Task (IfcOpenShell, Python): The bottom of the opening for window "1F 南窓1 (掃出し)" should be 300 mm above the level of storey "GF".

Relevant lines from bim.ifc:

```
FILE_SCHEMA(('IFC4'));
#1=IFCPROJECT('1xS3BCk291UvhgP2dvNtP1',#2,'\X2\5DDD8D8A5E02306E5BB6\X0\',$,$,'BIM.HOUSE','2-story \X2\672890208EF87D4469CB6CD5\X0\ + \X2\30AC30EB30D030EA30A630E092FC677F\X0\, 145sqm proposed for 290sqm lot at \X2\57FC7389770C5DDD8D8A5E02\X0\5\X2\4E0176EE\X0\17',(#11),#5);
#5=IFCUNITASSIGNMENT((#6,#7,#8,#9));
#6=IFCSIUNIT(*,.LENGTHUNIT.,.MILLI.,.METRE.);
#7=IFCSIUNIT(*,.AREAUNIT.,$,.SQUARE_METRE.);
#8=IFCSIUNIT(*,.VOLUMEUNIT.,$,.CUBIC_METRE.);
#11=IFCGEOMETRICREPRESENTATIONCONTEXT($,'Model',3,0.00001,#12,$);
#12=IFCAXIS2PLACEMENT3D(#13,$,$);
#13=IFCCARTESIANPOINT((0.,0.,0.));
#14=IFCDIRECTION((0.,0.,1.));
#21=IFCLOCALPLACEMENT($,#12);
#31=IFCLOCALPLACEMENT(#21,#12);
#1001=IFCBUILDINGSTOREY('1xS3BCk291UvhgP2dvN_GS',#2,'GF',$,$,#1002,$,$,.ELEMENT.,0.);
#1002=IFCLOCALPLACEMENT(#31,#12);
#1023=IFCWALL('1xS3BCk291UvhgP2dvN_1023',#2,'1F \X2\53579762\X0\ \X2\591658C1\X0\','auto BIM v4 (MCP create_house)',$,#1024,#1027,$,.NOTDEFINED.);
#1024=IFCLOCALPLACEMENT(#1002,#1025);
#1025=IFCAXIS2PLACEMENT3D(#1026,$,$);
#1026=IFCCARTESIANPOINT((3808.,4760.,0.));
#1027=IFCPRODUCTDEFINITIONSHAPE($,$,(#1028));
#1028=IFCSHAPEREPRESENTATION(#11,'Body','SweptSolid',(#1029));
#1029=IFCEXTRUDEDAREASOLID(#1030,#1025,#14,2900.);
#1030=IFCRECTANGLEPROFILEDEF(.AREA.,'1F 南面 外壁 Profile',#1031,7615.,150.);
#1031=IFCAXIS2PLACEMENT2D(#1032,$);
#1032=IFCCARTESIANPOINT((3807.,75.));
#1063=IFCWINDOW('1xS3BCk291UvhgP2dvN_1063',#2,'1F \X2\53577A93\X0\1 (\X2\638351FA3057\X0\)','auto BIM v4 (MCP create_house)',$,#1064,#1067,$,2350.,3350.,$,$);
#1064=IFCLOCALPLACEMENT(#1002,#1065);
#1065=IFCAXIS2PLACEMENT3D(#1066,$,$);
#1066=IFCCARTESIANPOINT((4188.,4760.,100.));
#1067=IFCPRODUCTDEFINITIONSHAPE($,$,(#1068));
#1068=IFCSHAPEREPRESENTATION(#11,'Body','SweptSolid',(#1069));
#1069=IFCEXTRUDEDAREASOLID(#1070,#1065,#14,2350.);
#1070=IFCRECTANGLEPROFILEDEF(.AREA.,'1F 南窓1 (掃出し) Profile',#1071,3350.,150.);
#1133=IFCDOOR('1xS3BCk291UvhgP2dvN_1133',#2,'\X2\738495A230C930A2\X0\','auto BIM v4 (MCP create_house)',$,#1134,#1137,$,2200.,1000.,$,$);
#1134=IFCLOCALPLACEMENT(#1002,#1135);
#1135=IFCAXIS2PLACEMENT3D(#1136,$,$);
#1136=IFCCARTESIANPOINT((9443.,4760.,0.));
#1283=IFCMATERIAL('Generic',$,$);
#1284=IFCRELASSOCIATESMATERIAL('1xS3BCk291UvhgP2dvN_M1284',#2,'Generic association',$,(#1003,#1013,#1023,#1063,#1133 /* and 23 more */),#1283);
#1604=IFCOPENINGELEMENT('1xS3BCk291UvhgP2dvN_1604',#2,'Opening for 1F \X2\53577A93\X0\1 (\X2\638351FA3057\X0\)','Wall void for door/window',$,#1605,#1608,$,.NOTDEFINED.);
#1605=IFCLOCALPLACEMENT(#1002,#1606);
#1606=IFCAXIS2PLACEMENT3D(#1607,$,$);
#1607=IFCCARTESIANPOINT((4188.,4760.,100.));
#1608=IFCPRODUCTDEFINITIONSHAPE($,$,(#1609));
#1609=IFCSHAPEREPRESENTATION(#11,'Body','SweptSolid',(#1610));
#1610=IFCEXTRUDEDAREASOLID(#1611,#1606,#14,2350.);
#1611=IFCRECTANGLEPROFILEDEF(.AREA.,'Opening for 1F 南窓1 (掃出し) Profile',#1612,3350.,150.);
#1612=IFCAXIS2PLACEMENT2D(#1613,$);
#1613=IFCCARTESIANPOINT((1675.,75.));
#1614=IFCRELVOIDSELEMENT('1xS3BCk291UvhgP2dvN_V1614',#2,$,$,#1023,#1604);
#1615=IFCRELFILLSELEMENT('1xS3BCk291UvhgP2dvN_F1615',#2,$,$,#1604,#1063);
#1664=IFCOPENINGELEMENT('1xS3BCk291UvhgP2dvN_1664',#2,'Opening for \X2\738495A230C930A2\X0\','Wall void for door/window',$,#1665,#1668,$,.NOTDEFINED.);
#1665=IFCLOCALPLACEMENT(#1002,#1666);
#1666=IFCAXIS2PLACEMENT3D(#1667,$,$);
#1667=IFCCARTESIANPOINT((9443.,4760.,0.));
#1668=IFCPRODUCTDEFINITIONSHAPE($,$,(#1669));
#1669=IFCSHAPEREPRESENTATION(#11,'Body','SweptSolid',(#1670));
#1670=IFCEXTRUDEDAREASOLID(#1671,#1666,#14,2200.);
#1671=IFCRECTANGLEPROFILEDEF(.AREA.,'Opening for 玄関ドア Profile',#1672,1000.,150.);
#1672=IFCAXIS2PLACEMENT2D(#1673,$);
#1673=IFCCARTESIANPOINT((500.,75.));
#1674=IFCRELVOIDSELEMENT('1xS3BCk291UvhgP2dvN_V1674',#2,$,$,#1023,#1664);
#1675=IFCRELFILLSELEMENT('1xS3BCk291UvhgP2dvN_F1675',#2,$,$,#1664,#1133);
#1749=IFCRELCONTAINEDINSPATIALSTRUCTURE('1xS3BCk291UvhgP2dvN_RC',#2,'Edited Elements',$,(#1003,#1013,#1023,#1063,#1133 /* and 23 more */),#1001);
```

```python
import numpy as np
import ifcopenshell
import ifcopenshell.api.geometry
import ifcopenshell.geom
import ifcopenshell.util.element
import ifcopenshell.util.placement
import ifcopenshell.util.shape
import ifcopenshell.util.unit

model = ifcopenshell.open("bim.ifc")
unit_scale = ifcopenshell.util.unit.calculate_unit_scale(model)

window = model.by_guid("1xS3BCk291UvhgP2dvN_1063")
opening = window.FillsVoids[0].RelatingOpeningElement
storey = ifcopenshell.util.element.get_container(window, ifc_class="IfcBuildingStorey")
level = ifcopenshell.util.placement.get_local_placement(storey.ObjectPlacement)[2, 3]

# The opening's origin need not be at the sill, so measure its lowest point.
shape = ifcopenshell.geom.create_shape(ifcopenshell.geom.settings(), opening)
bottom = ifcopenshell.util.shape.get_shape_bottom_elevation(shape, shape.geometry) / unit_scale
dz = level + 300.0 - bottom

shift = np.array([0.0, 0.0, dz])
# The window is not placed relative to its opening, so move both.
for product in (opening, window):
    matrix = ifcopenshell.util.placement.get_local_placement(product.ObjectPlacement)
    matrix[:3, 3] += shift
    ifcopenshell.api.geometry.edit_object_placement(model, product=product, matrix=matrix, is_si=False)

print(f"moved by {dz * unit_scale:+.3f} m")

model.write("bim_edited.ifc")
```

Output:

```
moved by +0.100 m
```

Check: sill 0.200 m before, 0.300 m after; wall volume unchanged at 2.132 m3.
